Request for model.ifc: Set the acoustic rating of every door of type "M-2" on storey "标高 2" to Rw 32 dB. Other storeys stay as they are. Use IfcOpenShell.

First a look at what the model holds.

```python
import ifcopenshell
import ifcopenshell.util.element

model = ifcopenshell.open("model.ifc")
print(model.schema)
storey = next(s for s in model.by_type("IfcBuildingStorey") if s.Name == "标高 2")
doors = [e for e in ifcopenshell.util.element.get_decomposition(storey) if e.is_a("IfcDoor")]
seen = {}
for e in doors:
    element_type = ifcopenshell.util.element.get_type(e)
    key = (element_type.Name if element_type != e and element_type else None, ifcopenshell.util.element.get_pset(e, "Pset_DoorCommon", "AcousticRating"))
    seen[key] = seen.get(key, 0) + 1
for (name, value), count in sorted(seen.items(), key=str):
    print(count, "x", name, "|", value)
```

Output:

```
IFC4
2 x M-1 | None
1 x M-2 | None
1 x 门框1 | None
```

```python
import ifcopenshell
import ifcopenshell.api.pset
import ifcopenshell.util.element

model = ifcopenshell.open("model.ifc")

storey = next(s for s in model.by_type("IfcBuildingStorey") if s.Name == "标高 2")
doors = [e for e in ifcopenshell.util.element.get_decomposition(storey) if e.is_a("IfcDoor")]

count = 0
for e in doors:
    element_type = ifcopenshell.util.element.get_type(e)
    if element_type in (None, e) or element_type.Name != "M-2":
        continue
    # add_pset returns the element's existing set when there is one.
    pset = ifcopenshell.api.pset.add_pset(model, product=e, name="Pset_DoorCommon")
    ifcopenshell.api.pset.edit_pset(model, pset=pset, properties={"AcousticRating": "Rw 32 dB"})
    count += 1

print(count, "doors updated")

model.write("model_updated.ifc")
```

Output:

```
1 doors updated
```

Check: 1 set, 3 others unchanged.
